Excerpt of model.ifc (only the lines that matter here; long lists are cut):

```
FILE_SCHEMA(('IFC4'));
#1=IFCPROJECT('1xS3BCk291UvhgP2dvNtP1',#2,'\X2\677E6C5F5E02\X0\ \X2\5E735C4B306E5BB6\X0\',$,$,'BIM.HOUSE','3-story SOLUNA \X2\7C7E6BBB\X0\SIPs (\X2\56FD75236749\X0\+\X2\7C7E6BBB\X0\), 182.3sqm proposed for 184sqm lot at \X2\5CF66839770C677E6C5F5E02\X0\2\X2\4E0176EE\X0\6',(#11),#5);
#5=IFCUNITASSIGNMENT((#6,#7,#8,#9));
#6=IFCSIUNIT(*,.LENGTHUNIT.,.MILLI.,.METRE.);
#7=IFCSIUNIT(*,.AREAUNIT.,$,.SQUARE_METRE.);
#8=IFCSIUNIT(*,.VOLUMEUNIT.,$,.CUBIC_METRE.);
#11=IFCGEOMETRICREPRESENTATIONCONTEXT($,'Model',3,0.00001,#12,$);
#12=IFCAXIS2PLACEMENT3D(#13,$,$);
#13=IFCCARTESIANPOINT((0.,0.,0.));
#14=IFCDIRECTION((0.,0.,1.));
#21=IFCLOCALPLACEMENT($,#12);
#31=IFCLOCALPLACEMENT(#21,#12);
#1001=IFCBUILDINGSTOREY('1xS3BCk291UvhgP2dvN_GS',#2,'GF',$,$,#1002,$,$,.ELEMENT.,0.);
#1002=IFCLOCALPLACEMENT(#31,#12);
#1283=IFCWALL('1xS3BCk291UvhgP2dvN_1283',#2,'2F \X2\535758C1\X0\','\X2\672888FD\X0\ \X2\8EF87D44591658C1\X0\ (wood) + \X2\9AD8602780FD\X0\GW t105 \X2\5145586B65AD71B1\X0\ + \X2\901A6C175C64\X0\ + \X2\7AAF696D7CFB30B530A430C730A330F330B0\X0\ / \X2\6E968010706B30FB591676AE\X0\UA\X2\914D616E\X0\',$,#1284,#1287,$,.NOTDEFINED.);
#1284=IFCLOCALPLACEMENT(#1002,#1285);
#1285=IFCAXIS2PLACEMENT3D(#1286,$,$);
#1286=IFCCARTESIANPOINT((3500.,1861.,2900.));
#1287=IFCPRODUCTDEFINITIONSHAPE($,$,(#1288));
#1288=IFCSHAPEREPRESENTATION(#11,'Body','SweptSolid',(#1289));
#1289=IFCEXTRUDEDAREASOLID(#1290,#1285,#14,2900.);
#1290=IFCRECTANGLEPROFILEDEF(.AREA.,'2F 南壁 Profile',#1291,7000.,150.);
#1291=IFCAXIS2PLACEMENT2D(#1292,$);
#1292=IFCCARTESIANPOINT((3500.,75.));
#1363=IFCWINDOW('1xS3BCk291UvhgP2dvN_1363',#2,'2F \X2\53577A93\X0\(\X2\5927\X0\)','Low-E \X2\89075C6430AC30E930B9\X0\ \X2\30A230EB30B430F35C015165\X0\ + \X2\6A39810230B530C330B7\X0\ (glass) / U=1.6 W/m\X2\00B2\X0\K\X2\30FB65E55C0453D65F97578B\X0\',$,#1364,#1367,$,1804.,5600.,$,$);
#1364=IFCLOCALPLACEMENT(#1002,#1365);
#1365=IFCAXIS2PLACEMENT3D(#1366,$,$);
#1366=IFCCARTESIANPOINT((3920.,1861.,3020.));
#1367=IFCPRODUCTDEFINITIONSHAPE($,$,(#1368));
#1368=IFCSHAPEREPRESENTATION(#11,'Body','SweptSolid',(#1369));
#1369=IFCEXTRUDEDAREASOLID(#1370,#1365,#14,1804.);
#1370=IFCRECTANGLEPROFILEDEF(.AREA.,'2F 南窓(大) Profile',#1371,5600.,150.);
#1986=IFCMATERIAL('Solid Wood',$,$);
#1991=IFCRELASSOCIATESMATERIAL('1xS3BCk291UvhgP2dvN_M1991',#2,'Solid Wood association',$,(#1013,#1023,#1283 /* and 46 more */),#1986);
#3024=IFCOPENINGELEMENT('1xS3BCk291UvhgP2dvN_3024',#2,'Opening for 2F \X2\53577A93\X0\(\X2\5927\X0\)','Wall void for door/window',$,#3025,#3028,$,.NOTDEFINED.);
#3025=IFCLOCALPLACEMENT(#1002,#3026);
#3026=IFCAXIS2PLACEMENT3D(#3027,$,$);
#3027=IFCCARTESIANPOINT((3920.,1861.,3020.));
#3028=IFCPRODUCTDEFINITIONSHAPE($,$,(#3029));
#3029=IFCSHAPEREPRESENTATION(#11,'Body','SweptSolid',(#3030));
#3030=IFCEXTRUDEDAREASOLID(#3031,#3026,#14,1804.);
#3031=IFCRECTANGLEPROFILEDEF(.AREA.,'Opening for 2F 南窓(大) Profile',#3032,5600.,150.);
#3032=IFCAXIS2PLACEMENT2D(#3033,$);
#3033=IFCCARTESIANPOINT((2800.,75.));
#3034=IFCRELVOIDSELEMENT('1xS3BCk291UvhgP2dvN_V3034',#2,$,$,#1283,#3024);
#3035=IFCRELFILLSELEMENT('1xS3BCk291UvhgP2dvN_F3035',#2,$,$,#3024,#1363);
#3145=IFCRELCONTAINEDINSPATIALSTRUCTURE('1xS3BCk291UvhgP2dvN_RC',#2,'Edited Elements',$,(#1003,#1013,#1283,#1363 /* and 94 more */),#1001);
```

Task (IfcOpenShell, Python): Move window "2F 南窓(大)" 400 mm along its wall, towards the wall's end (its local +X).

```python
import ifcopenshell
import ifcopenshell.api.geometry
import ifcopenshell.util.placement
import ifcopenshell.util.unit

model = ifcopenshell.open("model.ifc")
unit_scale = ifcopenshell.util.unit.calculate_unit_scale(model)

window = model.by_guid("1xS3BCk291UvhgP2dvN_1363")
opening = window.FillsVoids[0].RelatingOpeningElement
wall = opening.VoidsElements[0].RelatingBuildingElement

wall_matrix = ifcopenshell.util.placement.get_local_placement(wall.ObjectPlacement)
shift = wall_matrix[:3, 0] * 0.4 / unit_scale
before = ifcopenshell.util.placement.get_local_placement(window.ObjectPlacement)[:3, 3].copy()

# The window is not placed relative to its opening, so move both.
for product in (opening, window):
    matrix = ifcopenshell.util.placement.get_local_placement(product.ObjectPlacement)
    matrix[:3, 3] += shift
    ifcopenshell.api.geometry.edit_object_placement(model, product=product, matrix=matrix, is_si=False)

after = ifcopenshell.util.placement.get_local_placement(window.ObjectPlacement)[:3, 3]
print("window moved by", (after - before).round(3) + 0.0)

model.write("model-out.ifc")
```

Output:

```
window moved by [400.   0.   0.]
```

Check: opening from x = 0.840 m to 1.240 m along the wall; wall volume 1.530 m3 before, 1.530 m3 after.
